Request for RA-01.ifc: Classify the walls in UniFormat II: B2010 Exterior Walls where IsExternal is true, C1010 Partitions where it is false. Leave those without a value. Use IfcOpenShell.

First a look at what the model holds.

```python
import ifcopenshell
import ifcopenshell.util.element

model = ifcopenshell.open("RA-01.ifc")
print(model.schema)
print("classifications:", [c.Name for c in model.by_type("IfcClassification")])
values = [ifcopenshell.util.element.get_pset(e, "Pset_WallCommon", "IsExternal") for e in model.by_type("IfcWall")]
for value in (True, False, None):
    print("IsExternal", value, values.count(value))
```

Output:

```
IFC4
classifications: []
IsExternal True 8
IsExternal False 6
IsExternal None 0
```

```python
import ifcopenshell
import ifcopenshell.api.classification
import ifcopenshell.util.element

model = ifcopenshell.open("RA-01.ifc")

system = ifcopenshell.api.classification.add_classification(model, classification="UniFormat II")

walls = model.by_type("IfcWall")
external = {e: ifcopenshell.util.element.get_pset(e, "Pset_WallCommon", "IsExternal") for e in walls}
for flag, code, name in ((True, "B2010", "Exterior Walls"), (False, "C1010", "Partitions")):
    products = [e for e in walls if external[e] is flag]
    ifcopenshell.api.classification.add_reference(
        model, products=products, classification=system, identification=code, name=name
    )
    print(code, len(products))

model.write("RA-01_updated.ifc")
```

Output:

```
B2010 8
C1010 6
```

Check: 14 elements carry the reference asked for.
